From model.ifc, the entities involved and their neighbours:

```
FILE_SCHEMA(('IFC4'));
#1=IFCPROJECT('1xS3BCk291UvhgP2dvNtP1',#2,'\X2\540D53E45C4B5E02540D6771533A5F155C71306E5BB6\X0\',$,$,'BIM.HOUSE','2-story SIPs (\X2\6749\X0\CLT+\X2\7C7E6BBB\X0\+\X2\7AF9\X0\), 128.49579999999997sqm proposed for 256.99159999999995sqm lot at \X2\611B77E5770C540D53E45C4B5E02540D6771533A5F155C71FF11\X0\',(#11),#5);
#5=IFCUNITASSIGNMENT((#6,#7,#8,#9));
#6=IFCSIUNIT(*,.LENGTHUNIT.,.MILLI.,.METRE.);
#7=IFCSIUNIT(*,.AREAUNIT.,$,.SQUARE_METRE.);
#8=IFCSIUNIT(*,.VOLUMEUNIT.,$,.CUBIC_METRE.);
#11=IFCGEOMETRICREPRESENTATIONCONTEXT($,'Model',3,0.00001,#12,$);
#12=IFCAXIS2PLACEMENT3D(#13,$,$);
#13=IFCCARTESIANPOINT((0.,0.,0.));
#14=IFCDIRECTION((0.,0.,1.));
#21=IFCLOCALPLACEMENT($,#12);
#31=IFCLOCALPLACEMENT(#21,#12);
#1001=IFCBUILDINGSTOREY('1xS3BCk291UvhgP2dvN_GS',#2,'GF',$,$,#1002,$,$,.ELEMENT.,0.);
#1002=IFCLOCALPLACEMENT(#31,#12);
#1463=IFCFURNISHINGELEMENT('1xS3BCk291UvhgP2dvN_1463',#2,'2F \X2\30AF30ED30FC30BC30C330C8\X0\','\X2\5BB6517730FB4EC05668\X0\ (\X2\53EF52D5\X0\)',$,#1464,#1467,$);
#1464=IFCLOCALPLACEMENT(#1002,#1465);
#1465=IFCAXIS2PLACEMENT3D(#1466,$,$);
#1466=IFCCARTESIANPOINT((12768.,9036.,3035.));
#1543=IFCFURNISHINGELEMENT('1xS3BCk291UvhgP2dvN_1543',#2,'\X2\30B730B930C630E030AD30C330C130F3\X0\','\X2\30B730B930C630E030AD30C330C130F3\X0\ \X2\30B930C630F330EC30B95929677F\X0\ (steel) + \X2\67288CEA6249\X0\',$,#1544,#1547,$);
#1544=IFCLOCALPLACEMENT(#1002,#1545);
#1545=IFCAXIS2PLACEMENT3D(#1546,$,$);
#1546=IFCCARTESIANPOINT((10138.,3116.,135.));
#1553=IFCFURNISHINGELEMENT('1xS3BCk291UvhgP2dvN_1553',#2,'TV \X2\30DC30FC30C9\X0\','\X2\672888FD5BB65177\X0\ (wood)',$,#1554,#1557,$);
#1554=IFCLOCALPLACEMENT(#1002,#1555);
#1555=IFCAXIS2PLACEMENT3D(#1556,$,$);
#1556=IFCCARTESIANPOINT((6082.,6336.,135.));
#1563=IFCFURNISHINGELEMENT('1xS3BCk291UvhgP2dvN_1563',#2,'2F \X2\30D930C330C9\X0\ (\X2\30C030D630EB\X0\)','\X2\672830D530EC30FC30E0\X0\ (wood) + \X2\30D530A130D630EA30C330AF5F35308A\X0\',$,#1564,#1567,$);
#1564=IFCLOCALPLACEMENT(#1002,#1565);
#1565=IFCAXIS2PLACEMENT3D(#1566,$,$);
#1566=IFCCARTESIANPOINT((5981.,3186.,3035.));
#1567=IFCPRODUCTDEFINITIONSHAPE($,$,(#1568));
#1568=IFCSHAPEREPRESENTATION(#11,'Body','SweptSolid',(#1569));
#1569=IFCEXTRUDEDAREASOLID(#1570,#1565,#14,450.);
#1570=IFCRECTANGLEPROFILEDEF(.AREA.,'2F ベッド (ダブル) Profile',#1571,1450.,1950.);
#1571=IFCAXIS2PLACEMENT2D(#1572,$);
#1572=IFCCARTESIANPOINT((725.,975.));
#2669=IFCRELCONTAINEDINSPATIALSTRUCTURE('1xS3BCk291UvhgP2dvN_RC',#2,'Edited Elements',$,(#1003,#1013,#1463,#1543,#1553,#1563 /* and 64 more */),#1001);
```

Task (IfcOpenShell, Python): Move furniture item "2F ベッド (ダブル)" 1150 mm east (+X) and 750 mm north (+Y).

```python
import ifcopenshell
import ifcopenshell.api.geometry
import ifcopenshell.util.placement

model = ifcopenshell.open("model.ifc")

item = model.by_guid("1xS3BCk291UvhgP2dvN_1563")
matrix = ifcopenshell.util.placement.get_local_placement(item.ObjectPlacement)
matrix[0, 3] += 1150.0
matrix[1, 3] += 750.0
ifcopenshell.api.geometry.edit_object_placement(model, product=item, matrix=matrix, is_si=False)

print(ifcopenshell.util.placement.get_local_placement(item.ObjectPlacement).round(3) + 0.0)

model.write("model-out.ifc")
```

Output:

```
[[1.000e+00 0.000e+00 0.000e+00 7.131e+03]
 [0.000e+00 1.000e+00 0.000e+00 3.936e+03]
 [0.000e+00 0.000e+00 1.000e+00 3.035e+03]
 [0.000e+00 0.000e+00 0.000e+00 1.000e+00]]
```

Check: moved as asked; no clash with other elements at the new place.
